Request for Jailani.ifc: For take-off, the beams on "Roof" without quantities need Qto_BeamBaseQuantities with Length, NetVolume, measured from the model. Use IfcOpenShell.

First a look at what the model holds.

```python
import ifcopenshell
import ifcopenshell.util.element
import ifcopenshell.util.unit

model = ifcopenshell.open("Jailani.ifc")
print(model.schema)
for unit_type in ("LENGTHUNIT", "AREAUNIT", "VOLUMEUNIT"):
    print(unit_type, ifcopenshell.util.unit.calculate_unit_scale(model, unit_type))
storey = next(s for s in model.by_type("IfcBuildingStorey") if s.Name == "Roof")
beams = [e for e in ifcopenshell.util.element.get_decomposition(storey) if e.is_a("IfcBeam")]
for e in sorted(beams, key=lambda e: e.id()):
    print(e.id(), e.is_a(), e.Name, list(ifcopenshell.util.element.get_psets(e, qtos_only=True)), sep=" | ")
```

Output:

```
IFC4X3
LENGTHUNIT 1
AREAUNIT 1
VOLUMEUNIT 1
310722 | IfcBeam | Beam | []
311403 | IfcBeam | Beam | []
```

```python
import ifcopenshell
import ifcopenshell.api.pset
import ifcopenshell.geom
import ifcopenshell.util.element
import ifcopenshell.util.shape
import ifcopenshell.util.unit

model = ifcopenshell.open("Jailani.ifc")
unit_scale = ifcopenshell.util.unit.calculate_unit_scale(model)
volume_scale = ifcopenshell.util.unit.calculate_unit_scale(model, "VOLUMEUNIT")
settings = ifcopenshell.geom.settings()

storey = next(s for s in model.by_type("IfcBuildingStorey") if s.Name == "Roof")
beams = [e for e in ifcopenshell.util.element.get_decomposition(storey) if e.is_a("IfcBeam")]

for e in sorted(beams, key=lambda e: e.id()):
    if ifcopenshell.util.element.get_psets(e, qtos_only=True, should_inherit=False):
        continue
    # Geometry comes back in metres, in the element's own axes.
    shape = ifcopenshell.geom.create_shape(settings, e)
    values = {
        "Length": ifcopenshell.util.shape.get_max_xyz(shape.geometry) / unit_scale,
        "NetVolume": ifcopenshell.util.shape.get_volume(shape.geometry) / volume_scale,
    }
    qto = ifcopenshell.api.pset.add_qto(model, product=e, name="Qto_BeamBaseQuantities")
    ifcopenshell.api.pset.edit_qto(model, qto=qto, properties=values)
    print(e.id(), {k: round(v, 3) for k, v in values.items()})

model.write("Jailani_rev.ifc")
```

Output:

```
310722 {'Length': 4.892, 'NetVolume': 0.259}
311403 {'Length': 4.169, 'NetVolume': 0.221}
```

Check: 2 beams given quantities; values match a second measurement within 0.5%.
